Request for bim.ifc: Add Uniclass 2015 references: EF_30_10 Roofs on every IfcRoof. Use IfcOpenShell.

First a look at what the model holds.

```python
import ifcopenshell

model = ifcopenshell.open("bim.ifc")
print(model.schema)
print("classifications:", [c.Name for c in model.by_type("IfcClassification")])
for ifc_class in ("IfcDoor", "IfcRoof", "IfcStair", "IfcWall", "IfcWindow"):
    print(ifc_class, len(model.by_type(ifc_class)))
```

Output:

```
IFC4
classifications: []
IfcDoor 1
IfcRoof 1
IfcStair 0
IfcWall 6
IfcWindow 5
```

```python
import ifcopenshell
import ifcopenshell.api.classification

model = ifcopenshell.open("bim.ifc")

system = ifcopenshell.api.classification.add_classification(model, classification="Uniclass 2015")

codes = {
    "IfcRoof": ("EF_30_10", "Roofs"),
}
for ifc_class, (code, name) in codes.items():
    products = model.by_type(ifc_class)
    ifcopenshell.api.classification.add_reference(
        model, products=products, classification=system, identification=code, name=name
    )
    print(code, len(products))

model.write("bim_v2.ifc")
```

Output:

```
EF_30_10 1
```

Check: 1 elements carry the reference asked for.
